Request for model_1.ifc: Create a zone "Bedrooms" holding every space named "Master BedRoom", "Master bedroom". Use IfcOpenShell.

First a look at what the model holds.

```python
import ifcopenshell

model = ifcopenshell.open("model_1.ifc")
print(model.schema)
seen = {}
for space in model.by_type("IfcSpace"):
    seen[space.LongName] = seen.get(space.LongName, 0) + 1
for name, count in sorted(seen.items(), key=str):
    print(count, "x", name)
print("zones:", [z.Name for z in model.by_type("IfcZone")][:20])
```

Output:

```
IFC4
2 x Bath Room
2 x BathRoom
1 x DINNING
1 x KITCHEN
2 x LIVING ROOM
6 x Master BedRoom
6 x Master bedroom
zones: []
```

```python
import ifcopenshell
import ifcopenshell.api.group
import ifcopenshell.api.root

model = ifcopenshell.open("model_1.ifc")

names = {"Master BedRoom", "Master bedroom"}
spaces = [s for s in model.by_type("IfcSpace") if s.LongName in names]

zone = ifcopenshell.api.root.create_entity(model, ifc_class="IfcZone", name="Bedrooms")
ifcopenshell.api.group.assign_group(model, products=spaces, group=zone)
print(len(spaces), "spaces in", zone.Name)

model.write("model_1_updated.ifc")
```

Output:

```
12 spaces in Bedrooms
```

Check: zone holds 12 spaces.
